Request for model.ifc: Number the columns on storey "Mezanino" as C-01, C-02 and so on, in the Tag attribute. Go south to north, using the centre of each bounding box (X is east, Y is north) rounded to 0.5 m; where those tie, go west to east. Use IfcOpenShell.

First a look at what the model holds.

```python
import ifcopenshell
import ifcopenshell.util.element
import ifcopenshell.util.placement

model = ifcopenshell.open("model.ifc")
print(model.schema)
storey = next(s for s in model.by_type("IfcBuildingStorey") if s.Name == "Mezanino")
columns = [e for e in ifcopenshell.util.element.get_decomposition(storey) if e.is_a("IfcColumn")]
for e in sorted(columns, key=lambda e: e.id()):
    origin = ifcopenshell.util.placement.get_local_placement(e.ObjectPlacement)[:3, 3]
    print(e.id(), e.Tag, e.Name, origin.round(2) + 0.0, sep=" | ")
```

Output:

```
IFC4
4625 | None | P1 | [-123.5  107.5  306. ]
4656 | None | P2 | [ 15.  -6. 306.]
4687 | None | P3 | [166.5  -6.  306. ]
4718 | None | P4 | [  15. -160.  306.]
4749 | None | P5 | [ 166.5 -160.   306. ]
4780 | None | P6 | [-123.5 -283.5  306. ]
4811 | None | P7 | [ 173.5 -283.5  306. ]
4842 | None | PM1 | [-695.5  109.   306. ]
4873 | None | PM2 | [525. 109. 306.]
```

```python
import ifcopenshell
import ifcopenshell.geom
import ifcopenshell.util.element
import ifcopenshell.util.shape

model = ifcopenshell.open("model.ifc")
settings = ifcopenshell.geom.settings()
settings.set("use-world-coords", True)


def centre(element):
    shape = ifcopenshell.geom.create_shape(settings, element)
    return ifcopenshell.util.shape.get_bbox_centroid(shape.geometry)


storey = next(s for s in model.by_type("IfcBuildingStorey") if s.Name == "Mezanino")
columns = [e for e in ifcopenshell.util.element.get_decomposition(storey) if e.is_a("IfcColumn")]

# Insertion points can sit at a corner or the storey origin, so sort by the geometry (in metres).
centres = {e: centre(e) for e in columns}
columns.sort(key=lambda e: (round(centres[e][1] / 0.5), centres[e][0]))

for i, e in enumerate(columns, start=1):
    number = f"C-{i:02d}"
    e.Tag = number
    print(e.id(), number)

model.write("model_updated.ifc")
```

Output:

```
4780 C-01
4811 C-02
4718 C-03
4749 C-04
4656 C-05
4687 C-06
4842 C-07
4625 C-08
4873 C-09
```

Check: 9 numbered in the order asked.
